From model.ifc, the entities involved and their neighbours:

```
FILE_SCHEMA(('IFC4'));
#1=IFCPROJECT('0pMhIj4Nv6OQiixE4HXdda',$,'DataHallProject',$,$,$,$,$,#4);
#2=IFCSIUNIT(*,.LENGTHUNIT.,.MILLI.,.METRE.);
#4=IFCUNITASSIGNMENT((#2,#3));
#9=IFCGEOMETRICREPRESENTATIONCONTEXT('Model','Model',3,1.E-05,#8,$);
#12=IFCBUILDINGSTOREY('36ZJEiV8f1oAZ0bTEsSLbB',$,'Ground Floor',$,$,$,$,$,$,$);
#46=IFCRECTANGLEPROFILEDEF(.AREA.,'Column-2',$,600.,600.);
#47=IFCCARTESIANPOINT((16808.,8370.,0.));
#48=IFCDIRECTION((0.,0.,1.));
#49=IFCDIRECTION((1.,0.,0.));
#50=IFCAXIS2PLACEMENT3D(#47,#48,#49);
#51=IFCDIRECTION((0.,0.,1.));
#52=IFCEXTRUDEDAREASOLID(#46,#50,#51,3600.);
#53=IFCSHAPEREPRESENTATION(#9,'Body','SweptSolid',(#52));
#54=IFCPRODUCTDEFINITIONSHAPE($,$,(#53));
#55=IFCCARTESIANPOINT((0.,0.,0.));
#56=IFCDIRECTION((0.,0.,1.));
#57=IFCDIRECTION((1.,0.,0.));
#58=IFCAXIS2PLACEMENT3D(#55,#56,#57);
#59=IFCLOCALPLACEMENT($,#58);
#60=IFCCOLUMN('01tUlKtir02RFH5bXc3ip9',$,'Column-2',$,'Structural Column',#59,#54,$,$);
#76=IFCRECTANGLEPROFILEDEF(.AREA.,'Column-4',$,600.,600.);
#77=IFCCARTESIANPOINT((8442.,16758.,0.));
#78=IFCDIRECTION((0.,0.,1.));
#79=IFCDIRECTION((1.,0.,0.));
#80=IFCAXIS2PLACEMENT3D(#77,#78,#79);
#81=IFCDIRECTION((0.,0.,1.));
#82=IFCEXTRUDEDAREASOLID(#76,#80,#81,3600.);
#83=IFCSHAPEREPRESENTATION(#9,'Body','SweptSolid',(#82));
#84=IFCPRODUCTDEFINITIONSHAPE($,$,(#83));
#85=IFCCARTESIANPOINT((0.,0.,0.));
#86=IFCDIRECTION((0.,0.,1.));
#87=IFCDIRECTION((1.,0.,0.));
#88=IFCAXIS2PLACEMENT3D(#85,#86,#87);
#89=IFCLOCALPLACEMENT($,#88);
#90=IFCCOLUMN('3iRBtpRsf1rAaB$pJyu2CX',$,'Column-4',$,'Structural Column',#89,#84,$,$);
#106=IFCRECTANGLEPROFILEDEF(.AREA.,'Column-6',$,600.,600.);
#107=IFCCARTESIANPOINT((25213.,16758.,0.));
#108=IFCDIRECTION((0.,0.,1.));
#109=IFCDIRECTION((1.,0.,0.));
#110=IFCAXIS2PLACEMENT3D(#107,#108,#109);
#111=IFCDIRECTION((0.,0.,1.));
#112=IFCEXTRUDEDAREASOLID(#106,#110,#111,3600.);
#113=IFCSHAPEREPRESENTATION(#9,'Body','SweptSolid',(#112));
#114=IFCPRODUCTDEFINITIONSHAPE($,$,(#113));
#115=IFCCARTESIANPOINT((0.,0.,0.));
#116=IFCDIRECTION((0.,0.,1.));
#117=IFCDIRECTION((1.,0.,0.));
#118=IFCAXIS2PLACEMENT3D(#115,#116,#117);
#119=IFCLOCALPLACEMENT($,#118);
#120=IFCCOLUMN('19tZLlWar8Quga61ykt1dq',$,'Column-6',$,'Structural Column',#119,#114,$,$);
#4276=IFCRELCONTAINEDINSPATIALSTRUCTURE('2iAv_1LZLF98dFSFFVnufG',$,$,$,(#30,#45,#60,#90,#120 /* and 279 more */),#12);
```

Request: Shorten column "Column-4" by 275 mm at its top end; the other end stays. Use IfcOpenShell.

```python
import ifcopenshell
import ifcopenshell.util.unit

model = ifcopenshell.open("model.ifc")
unit_scale = ifcopenshell.util.unit.calculate_unit_scale(model)

member = model.by_id(90)
change = -0.275 / unit_scale

# The extrusion runs towards the end named, so only its depth changes.
body = next(r for r in member.Representation.Representations if r.RepresentationIdentifier == "Body")
solid = body.Items[0]
old_length = solid.Depth
solid.Depth += change

print(f"length {old_length:g} -> {solid.Depth:g}")

model.write("model_edited.ifc")
```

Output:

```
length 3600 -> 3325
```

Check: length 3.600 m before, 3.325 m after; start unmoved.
